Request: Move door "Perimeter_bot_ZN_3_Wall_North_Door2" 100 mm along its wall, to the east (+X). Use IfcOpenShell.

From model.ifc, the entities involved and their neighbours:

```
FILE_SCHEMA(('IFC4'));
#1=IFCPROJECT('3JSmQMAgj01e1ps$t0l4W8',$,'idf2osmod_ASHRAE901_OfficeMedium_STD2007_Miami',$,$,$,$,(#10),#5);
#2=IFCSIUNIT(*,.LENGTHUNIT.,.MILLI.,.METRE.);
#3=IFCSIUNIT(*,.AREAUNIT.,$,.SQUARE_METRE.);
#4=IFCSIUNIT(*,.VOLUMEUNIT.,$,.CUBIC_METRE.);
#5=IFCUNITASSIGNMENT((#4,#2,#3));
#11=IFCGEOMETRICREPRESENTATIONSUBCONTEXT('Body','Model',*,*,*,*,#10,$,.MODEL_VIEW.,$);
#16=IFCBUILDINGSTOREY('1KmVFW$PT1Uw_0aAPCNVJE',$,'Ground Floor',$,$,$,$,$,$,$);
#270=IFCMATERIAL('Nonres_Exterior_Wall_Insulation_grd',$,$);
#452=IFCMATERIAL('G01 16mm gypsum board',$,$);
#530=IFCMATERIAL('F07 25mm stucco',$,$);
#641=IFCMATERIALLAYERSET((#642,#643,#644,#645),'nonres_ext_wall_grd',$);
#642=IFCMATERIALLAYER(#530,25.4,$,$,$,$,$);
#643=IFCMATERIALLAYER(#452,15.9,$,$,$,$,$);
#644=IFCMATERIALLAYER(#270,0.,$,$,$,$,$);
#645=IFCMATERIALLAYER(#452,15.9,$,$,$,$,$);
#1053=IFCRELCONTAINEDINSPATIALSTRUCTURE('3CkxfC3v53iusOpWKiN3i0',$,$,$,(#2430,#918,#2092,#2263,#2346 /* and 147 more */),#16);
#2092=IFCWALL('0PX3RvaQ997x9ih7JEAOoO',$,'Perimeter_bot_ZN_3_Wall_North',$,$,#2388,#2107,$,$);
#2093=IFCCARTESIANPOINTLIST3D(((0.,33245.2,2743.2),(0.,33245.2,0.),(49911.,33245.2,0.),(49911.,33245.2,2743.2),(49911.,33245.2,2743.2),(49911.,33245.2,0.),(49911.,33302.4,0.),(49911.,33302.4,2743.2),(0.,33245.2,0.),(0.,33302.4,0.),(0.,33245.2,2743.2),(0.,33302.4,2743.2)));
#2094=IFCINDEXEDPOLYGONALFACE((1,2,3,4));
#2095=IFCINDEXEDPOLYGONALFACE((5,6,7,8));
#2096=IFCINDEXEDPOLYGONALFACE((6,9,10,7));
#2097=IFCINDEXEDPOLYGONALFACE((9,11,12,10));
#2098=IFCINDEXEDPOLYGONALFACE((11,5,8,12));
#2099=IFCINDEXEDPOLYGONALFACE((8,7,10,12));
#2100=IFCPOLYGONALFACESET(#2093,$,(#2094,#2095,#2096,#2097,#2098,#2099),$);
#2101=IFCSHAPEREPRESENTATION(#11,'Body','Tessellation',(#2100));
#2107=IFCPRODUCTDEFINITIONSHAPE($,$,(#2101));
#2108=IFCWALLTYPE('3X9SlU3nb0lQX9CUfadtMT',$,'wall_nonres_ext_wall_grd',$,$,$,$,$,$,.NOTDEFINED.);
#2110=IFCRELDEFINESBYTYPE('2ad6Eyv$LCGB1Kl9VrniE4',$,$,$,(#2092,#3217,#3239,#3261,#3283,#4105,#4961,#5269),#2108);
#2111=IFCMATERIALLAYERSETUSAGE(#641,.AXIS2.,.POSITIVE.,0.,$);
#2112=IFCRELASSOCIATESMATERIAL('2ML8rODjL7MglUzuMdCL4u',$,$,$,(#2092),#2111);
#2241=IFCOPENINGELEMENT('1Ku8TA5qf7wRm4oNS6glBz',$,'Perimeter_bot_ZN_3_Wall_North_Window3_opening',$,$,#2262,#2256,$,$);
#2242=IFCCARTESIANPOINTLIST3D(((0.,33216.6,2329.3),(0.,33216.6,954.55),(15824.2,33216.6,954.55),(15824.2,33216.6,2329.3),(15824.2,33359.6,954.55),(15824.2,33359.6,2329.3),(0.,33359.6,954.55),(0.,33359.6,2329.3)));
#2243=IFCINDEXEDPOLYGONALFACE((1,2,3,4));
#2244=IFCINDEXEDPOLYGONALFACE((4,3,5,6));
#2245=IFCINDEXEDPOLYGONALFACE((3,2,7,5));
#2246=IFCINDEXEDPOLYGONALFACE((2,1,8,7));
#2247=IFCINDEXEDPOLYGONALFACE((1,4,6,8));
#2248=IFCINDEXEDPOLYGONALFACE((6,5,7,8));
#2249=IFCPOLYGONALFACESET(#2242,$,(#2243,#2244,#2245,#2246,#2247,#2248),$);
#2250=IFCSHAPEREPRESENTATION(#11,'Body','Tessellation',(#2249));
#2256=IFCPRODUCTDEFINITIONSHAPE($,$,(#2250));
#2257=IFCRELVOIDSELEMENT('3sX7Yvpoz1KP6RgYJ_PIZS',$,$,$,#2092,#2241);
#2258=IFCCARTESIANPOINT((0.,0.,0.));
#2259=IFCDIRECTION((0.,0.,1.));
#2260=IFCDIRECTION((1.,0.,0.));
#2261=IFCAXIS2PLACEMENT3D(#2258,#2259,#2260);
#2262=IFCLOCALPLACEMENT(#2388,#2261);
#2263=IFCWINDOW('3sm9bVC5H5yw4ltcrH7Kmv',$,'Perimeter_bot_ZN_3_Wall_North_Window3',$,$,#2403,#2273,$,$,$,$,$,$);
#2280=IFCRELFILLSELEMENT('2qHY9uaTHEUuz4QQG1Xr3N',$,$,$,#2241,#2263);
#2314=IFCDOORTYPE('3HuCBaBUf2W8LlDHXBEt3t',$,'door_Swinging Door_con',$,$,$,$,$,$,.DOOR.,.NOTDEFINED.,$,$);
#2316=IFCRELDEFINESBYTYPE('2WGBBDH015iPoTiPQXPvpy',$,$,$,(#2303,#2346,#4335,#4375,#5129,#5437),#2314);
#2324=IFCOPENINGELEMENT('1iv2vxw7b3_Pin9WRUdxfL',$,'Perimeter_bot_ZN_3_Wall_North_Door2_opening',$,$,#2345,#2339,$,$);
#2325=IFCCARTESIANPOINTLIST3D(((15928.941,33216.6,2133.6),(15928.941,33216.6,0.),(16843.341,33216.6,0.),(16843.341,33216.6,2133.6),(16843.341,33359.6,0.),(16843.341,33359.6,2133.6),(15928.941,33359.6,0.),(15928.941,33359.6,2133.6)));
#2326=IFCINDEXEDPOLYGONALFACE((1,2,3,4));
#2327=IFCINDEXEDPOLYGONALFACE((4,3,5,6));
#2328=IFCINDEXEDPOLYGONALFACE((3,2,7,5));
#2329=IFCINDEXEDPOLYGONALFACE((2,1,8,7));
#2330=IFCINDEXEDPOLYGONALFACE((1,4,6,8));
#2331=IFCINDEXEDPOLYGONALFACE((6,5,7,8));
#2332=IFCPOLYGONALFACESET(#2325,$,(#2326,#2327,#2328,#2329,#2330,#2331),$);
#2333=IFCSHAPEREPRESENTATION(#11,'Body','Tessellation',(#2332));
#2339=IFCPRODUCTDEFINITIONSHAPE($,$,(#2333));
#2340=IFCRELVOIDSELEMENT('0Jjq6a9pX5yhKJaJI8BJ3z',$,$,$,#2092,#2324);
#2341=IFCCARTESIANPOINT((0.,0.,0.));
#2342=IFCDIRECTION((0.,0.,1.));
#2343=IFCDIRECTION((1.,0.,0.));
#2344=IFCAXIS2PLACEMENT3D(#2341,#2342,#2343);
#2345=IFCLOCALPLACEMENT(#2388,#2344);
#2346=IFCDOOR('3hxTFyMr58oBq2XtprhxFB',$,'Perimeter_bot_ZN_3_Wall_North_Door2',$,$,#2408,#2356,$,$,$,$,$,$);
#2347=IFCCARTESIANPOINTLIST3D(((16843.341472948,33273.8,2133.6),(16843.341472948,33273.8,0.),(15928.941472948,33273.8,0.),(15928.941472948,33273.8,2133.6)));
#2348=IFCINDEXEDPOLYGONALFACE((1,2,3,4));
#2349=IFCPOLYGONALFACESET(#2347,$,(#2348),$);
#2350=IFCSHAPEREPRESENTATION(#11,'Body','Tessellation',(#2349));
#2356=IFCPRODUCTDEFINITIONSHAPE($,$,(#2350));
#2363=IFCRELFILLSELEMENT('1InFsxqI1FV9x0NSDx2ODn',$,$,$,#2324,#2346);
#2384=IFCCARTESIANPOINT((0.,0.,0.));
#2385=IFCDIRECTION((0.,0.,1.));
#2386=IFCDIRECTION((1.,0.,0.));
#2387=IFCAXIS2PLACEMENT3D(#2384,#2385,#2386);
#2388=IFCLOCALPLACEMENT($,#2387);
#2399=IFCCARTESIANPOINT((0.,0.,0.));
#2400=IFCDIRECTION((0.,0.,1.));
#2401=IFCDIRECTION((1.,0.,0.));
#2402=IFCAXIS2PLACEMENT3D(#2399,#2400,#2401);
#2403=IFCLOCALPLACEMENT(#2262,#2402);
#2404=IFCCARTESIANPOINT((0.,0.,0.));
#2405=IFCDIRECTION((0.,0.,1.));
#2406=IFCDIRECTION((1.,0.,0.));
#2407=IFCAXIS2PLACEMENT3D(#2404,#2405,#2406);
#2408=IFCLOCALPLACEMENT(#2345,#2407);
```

```python
import ifcopenshell
import ifcopenshell.api.geometry
import ifcopenshell.util.placement
import ifcopenshell.util.unit

model = ifcopenshell.open("model.ifc")
unit_scale = ifcopenshell.util.unit.calculate_unit_scale(model)

door = model.by_guid("3hxTFyMr58oBq2XtprhxFB")
opening = door.FillsVoids[0].RelatingOpeningElement
wall = opening.VoidsElements[0].RelatingBuildingElement

wall_matrix = ifcopenshell.util.placement.get_local_placement(wall.ObjectPlacement)
shift = wall_matrix[:3, 0] * 0.1 / unit_scale
before = ifcopenshell.util.placement.get_local_placement(door.ObjectPlacement)[:3, 3].copy()

# The door is placed relative to its opening, so it follows when the opening moves.
matrix = ifcopenshell.util.placement.get_local_placement(opening.ObjectPlacement)
matrix[:3, 3] += shift
ifcopenshell.api.geometry.edit_object_placement(
    model, product=opening, matrix=matrix, is_si=False, should_transform_children=True
)

after = ifcopenshell.util.placement.get_local_placement(door.ObjectPlacement)[:3, 3]
print("door moved by", (after - before).round(3) + 0.0)

model.write("model_edited.ifc")
```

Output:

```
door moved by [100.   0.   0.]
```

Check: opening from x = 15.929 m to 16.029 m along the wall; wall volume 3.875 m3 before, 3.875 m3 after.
